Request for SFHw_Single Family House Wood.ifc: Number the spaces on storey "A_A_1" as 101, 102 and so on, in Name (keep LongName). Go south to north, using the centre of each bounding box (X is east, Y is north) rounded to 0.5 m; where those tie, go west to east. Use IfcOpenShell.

First a look at what the model holds.

```python
import ifcopenshell
import ifcopenshell.util.element
import ifcopenshell.util.placement

model = ifcopenshell.open("SFHw_Single Family House Wood.ifc")
print(model.schema)
storey = next(s for s in model.by_type("IfcBuildingStorey") if s.Name == "A_A_1")
spaces = [e for e in ifcopenshell.util.element.get_decomposition(storey) if e.is_a("IfcSpace")]
for e in sorted(spaces, key=lambda e: e.id()):
    origin = ifcopenshell.util.placement.get_local_placement(e.ObjectPlacement)[:3, 3]
    print(e.id(), e.Name, e.LongName, origin.round(2) + 0.0, sep=" | ")
```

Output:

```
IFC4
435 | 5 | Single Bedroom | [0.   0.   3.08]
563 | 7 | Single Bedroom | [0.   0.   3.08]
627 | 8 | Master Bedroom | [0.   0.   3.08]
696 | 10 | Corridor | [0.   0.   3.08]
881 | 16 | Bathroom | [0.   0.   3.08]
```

```python
import ifcopenshell
import ifcopenshell.geom
import ifcopenshell.util.element
import ifcopenshell.util.shape

model = ifcopenshell.open("SFHw_Single Family House Wood.ifc")
settings = ifcopenshell.geom.settings()
settings.set("use-world-coords", True)


def centre(element):
    shape = ifcopenshell.geom.create_shape(settings, element)
    return ifcopenshell.util.shape.get_bbox_centroid(shape.geometry)


storey = next(s for s in model.by_type("IfcBuildingStorey") if s.Name == "A_A_1")
spaces = [e for e in ifcopenshell.util.element.get_decomposition(storey) if e.is_a("IfcSpace")]

# Insertion points can sit at a corner or the storey origin, so sort by the geometry (in metres).
centres = {e: centre(e) for e in spaces}
spaces.sort(key=lambda e: (round(centres[e][1] / 0.5), centres[e][0]))

for i, e in enumerate(spaces, start=1):
    number = f"1{i:02d}"
    e.Name = number
    print(e.id(), number)

model.write("SFHw_Single Family House Wood_edited.ifc")
```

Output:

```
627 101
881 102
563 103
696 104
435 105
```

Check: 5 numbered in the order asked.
